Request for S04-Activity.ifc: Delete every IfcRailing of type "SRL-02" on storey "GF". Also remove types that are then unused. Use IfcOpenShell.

First a look at what the model holds.

```python
import ifcopenshell
import ifcopenshell.util.element

model = ifcopenshell.open("S04-Activity.ifc")
print(model.schema)
storey = next(s for s in model.by_type("IfcBuildingStorey") if s.Name == "GF")
railings = [e for e in ifcopenshell.util.element.get_decomposition(storey) if e.is_a("IfcRailing")]
seen = {}
for e in railings:
    element_type = ifcopenshell.util.element.get_type(e)
    name = element_type.Name if element_type not in (None, e) else None
    seen[name] = seen.get(name, 0) + 1
for name, count in sorted(seen.items(), key=str):
    print(count, "x", name)
```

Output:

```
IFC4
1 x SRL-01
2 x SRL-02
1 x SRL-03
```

```python
import ifcopenshell
import ifcopenshell.api.root
import ifcopenshell.util.element

model = ifcopenshell.open("S04-Activity.ifc")

storey = next(s for s in model.by_type("IfcBuildingStorey") if s.Name == "GF")
railings = [e for e in ifcopenshell.util.element.get_decomposition(storey) if e.is_a("IfcRailing")]
targets = [e for e in railings if (t := ifcopenshell.util.element.get_type(e)) not in (None, e) and t.Name == "SRL-02"]
types = {ifcopenshell.util.element.get_type(e) for e in targets} - {None, *targets}

for e in targets:
    ifcopenshell.api.root.remove_product(model, product=e)
print(len(targets), "removed")

unused = [t for t in types if not ifcopenshell.util.element.get_types(t)]
for t in unused:
    ifcopenshell.api.root.remove_product(model, product=t)
print(len(unused), "unused types removed")

model.write("S04-Activity-out.ifc")
```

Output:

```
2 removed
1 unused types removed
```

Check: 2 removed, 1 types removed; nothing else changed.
